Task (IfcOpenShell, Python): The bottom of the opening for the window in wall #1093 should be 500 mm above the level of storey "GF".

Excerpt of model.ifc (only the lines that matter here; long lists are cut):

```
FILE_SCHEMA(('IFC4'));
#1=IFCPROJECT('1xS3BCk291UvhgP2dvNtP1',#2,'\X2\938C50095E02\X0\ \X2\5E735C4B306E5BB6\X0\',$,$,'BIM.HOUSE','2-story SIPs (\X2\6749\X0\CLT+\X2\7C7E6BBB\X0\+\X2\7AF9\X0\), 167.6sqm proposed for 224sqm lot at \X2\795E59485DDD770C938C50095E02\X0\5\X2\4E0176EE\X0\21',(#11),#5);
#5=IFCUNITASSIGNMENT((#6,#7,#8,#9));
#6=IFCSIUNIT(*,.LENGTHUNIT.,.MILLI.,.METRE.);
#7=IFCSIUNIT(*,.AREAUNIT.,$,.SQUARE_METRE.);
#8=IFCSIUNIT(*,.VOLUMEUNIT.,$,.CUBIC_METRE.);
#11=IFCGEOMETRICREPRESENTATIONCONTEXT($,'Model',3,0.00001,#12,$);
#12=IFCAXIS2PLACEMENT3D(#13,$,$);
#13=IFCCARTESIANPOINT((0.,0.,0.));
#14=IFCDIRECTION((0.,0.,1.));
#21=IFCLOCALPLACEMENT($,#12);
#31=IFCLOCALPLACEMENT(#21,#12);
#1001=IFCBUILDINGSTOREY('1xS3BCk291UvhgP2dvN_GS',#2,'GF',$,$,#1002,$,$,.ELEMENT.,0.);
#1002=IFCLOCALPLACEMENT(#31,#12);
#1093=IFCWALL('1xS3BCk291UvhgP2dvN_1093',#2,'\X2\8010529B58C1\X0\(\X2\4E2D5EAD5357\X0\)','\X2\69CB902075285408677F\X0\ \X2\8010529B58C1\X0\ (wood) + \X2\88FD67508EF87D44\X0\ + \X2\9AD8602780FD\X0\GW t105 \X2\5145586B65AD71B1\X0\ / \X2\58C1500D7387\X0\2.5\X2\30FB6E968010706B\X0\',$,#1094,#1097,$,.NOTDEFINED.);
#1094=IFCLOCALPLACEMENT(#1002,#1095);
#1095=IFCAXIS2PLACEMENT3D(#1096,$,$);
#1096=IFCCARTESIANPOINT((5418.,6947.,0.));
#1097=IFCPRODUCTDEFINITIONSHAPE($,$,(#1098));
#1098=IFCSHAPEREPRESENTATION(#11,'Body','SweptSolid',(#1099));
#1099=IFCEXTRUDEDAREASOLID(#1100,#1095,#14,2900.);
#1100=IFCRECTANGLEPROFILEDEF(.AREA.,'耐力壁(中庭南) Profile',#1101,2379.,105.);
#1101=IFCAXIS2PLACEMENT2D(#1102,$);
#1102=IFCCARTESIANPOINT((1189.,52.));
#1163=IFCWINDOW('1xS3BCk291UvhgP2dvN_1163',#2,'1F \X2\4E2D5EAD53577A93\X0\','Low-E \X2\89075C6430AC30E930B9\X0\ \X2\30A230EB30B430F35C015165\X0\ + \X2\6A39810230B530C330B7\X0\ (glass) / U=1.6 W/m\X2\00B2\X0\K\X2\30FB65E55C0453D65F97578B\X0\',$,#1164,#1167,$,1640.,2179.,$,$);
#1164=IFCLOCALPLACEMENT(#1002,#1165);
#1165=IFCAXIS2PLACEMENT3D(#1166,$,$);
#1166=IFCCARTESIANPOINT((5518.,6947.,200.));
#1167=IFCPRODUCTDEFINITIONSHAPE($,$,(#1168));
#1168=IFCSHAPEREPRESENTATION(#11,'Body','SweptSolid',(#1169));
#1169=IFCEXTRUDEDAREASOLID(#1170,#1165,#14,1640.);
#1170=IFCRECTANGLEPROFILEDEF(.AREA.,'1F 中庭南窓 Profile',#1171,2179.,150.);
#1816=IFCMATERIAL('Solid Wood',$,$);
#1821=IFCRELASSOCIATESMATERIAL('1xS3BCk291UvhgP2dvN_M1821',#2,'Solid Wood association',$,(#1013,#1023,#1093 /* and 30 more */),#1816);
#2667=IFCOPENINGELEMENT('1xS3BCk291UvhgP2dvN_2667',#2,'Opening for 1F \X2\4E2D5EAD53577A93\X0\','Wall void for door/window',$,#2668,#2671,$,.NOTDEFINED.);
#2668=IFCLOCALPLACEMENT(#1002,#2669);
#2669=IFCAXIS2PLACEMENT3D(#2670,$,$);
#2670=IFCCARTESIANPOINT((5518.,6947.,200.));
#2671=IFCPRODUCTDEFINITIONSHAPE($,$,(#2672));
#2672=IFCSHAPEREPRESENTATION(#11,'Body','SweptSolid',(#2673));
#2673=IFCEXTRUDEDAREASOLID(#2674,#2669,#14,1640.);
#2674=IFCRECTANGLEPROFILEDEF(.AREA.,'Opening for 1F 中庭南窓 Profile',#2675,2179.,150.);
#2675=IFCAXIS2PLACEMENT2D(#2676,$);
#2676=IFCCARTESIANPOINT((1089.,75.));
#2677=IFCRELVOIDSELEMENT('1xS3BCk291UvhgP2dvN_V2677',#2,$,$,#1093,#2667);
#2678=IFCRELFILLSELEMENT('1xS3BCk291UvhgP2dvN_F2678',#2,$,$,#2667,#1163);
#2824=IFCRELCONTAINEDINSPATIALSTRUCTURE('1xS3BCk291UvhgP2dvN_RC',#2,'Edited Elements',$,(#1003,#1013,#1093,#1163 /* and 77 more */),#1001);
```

```python
import numpy as np
import ifcopenshell
import ifcopenshell.api.geometry
import ifcopenshell.geom
import ifcopenshell.util.element
import ifcopenshell.util.placement
import ifcopenshell.util.shape
import ifcopenshell.util.unit

model = ifcopenshell.open("model.ifc")
unit_scale = ifcopenshell.util.unit.calculate_unit_scale(model)

window = model.by_guid("1xS3BCk291UvhgP2dvN_1163")
opening = window.FillsVoids[0].RelatingOpeningElement
storey = ifcopenshell.util.element.get_container(window, ifc_class="IfcBuildingStorey")
level = ifcopenshell.util.placement.get_local_placement(storey.ObjectPlacement)[2, 3]

# The opening's origin need not be at the sill, so measure its lowest point.
shape = ifcopenshell.geom.create_shape(ifcopenshell.geom.settings(), opening)
bottom = ifcopenshell.util.shape.get_shape_bottom_elevation(shape, shape.geometry) / unit_scale
dz = level + 0.5 / unit_scale - bottom

shift = np.array([0.0, 0.0, dz])
# The window is not placed relative to its opening, so move both.
for product in (opening, window):
    matrix = ifcopenshell.util.placement.get_local_placement(product.ObjectPlacement)
    matrix[:3, 3] += shift
    ifcopenshell.api.geometry.edit_object_placement(model, product=product, matrix=matrix, is_si=False)

print(f"moved by {dz * unit_scale:+.3f} m")

model.write("model_v2.ifc")
```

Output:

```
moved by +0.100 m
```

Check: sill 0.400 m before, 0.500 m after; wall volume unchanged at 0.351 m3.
